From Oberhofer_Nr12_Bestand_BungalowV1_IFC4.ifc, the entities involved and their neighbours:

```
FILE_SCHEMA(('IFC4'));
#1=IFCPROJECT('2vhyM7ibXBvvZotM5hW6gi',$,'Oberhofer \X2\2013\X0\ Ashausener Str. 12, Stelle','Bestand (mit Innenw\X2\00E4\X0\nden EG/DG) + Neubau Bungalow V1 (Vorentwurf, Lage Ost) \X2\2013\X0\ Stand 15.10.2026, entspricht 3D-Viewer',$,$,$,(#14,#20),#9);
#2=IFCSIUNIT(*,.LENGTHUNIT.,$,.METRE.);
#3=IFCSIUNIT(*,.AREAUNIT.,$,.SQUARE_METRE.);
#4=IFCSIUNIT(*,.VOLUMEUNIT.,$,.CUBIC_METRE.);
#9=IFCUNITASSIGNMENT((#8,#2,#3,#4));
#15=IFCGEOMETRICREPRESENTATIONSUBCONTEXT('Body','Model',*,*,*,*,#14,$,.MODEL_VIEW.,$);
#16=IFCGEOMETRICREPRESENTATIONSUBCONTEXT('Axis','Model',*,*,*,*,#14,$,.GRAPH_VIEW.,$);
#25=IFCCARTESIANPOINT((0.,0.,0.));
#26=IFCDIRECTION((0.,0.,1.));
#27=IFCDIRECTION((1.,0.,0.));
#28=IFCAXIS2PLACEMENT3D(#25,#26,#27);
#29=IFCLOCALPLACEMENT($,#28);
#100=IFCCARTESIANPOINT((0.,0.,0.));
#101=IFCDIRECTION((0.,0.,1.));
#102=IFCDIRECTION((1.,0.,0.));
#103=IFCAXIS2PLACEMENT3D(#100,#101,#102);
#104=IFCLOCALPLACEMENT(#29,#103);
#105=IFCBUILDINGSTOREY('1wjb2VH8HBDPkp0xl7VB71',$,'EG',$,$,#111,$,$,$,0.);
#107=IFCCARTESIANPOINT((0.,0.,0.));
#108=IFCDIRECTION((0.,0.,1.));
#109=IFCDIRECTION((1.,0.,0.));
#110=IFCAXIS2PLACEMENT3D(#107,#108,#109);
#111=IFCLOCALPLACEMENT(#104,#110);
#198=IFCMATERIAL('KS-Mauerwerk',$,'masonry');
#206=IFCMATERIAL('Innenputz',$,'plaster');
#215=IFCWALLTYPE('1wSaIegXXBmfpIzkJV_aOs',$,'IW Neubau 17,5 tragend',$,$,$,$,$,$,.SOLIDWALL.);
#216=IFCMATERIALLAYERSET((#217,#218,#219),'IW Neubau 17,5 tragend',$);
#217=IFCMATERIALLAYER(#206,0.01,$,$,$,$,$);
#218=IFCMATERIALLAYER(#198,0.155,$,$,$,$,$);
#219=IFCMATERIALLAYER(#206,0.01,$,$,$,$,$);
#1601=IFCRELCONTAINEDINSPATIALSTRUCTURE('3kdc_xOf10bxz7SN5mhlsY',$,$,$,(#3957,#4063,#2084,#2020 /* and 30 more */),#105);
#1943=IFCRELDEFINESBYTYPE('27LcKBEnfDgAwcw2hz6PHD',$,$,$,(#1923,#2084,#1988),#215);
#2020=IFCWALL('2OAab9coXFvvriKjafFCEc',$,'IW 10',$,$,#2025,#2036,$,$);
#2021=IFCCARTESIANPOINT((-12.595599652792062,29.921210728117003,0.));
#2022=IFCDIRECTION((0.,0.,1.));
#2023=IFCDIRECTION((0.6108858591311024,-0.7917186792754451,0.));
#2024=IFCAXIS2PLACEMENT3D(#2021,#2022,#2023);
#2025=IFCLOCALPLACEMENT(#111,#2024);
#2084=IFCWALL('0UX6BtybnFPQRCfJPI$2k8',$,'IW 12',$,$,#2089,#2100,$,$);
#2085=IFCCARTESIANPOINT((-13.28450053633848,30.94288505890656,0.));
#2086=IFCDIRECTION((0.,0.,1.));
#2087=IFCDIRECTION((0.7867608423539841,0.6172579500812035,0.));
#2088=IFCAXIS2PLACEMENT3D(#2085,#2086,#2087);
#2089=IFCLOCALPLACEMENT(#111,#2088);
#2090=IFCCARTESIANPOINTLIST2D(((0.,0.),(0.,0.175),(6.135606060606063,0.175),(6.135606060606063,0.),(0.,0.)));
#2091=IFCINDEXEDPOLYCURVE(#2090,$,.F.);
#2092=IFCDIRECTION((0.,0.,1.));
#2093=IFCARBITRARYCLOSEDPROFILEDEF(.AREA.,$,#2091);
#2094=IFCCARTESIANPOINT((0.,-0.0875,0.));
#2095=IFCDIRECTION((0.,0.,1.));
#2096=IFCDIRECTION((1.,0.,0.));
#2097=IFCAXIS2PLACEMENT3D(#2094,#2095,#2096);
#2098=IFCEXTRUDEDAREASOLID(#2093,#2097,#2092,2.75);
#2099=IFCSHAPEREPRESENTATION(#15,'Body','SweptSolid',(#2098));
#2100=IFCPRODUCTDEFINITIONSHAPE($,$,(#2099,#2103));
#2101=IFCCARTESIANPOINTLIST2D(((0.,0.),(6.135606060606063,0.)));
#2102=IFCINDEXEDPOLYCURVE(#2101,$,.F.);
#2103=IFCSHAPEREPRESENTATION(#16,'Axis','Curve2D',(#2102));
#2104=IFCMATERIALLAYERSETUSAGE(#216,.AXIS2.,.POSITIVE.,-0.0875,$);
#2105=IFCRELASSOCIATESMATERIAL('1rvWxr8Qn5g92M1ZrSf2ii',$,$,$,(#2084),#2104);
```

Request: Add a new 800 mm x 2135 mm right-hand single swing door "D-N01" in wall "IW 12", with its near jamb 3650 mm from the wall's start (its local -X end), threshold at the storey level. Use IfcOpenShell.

```python
import numpy as np
import ifcopenshell
import ifcopenshell.api.feature
import ifcopenshell.api.geometry
import ifcopenshell.api.root
import ifcopenshell.api.spatial
import ifcopenshell.geom
import ifcopenshell.util.element
import ifcopenshell.util.placement
import ifcopenshell.util.representation
import ifcopenshell.util.shape
import ifcopenshell.util.unit

model = ifcopenshell.open("Oberhofer_Nr12_Bestand_BungalowV1_IFC4.ifc")
unit_scale = ifcopenshell.util.unit.calculate_unit_scale(model)
settings = ifcopenshell.geom.settings()


def volume(element):
    """Net volume in cubic metres, openings subtracted."""
    shape = ifcopenshell.geom.create_shape(settings, element)
    return ifcopenshell.util.shape.get_volume(shape.geometry)


wall = model.by_id(2084)
storey = ifcopenshell.util.element.get_container(wall, ifc_class="IfcBuildingStorey")
context = ifcopenshell.util.representation.get_context(model, "Model", "Body", "MODEL_VIEW")
before = volume(wall)

width, height, from_end, sill = 0.8, 2.135, 3.65, 0.0  # metres

# The wall runs along its own X axis, and the end named is its -X end.
wall_shape = ifcopenshell.geom.create_shape(settings, wall)
x, y, z = ifcopenshell.util.shape.get_vertices(wall_shape.geometry).T
start = x.min() + from_end
face, thickness = float(y.min()), float(y.max() - y.min())
wall_matrix = ifcopenshell.util.placement.get_local_placement(wall.ObjectPlacement)
level = ifcopenshell.util.placement.get_local_placement(storey.ObjectPlacement)[2, 3]


def in_wall(x, y):
    """Placement at x, y metres in the wall's axes, at sill height."""
    matrix = wall_matrix.copy()
    matrix[:, 3] = wall_matrix @ np.array([x / unit_scale, y / unit_scale, 0.0, 1.0])
    matrix[2, 3] = level + sill / unit_scale
    return matrix


# Opening: a box that overshoots both wall faces by 50 mm.
opening = ifcopenshell.api.root.create_entity(model, ifc_class="IfcOpeningElement", predefined_type="OPENING")
box = ifcopenshell.api.geometry.add_wall_representation(
    model, context=context, length=width, height=height, thickness=thickness + 0.1
)
ifcopenshell.api.geometry.assign_representation(model, product=opening, representation=box)
ifcopenshell.api.geometry.edit_object_placement(model, product=opening, matrix=in_wall(start, face - 0.05), is_si=False)
ifcopenshell.api.feature.add_feature(model, feature=opening, element=wall)

door = ifcopenshell.api.root.create_entity(model, ifc_class="IfcDoor", name="D-N01", predefined_type="DOOR")
door.OverallWidth, door.OverallHeight = width / unit_scale, height / unit_scale
door.OperationType = "SINGLE_SWING_RIGHT"
body = ifcopenshell.api.geometry.add_door_representation(
    model,
    context=context,
    overall_width=door.OverallWidth,
    overall_height=door.OverallHeight,
    operation_type="SINGLE_SWING_RIGHT",
    lining_properties={"LiningDepth": thickness / unit_scale, "ThresholdDepth": thickness / unit_scale},
)
ifcopenshell.api.geometry.assign_representation(model, product=door, representation=body)
ifcopenshell.api.spatial.assign_container(model, products=[door], relating_structure=storey)
ifcopenshell.api.feature.add_filling(model, opening=opening, element=door)

# The lining spans the wall, so the door starts at the wall face.
ifcopenshell.api.geometry.edit_object_placement(model, product=door, matrix=in_wall(start, face), is_si=False)

after = volume(wall)

print(f"wall volume {before:.3f} -> {after:.3f} m3")

model.write("Oberhofer_Nr12_Bestand_BungalowV1_IFC4_v2.ifc")
```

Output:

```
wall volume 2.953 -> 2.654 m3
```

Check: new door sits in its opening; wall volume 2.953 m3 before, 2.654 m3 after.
